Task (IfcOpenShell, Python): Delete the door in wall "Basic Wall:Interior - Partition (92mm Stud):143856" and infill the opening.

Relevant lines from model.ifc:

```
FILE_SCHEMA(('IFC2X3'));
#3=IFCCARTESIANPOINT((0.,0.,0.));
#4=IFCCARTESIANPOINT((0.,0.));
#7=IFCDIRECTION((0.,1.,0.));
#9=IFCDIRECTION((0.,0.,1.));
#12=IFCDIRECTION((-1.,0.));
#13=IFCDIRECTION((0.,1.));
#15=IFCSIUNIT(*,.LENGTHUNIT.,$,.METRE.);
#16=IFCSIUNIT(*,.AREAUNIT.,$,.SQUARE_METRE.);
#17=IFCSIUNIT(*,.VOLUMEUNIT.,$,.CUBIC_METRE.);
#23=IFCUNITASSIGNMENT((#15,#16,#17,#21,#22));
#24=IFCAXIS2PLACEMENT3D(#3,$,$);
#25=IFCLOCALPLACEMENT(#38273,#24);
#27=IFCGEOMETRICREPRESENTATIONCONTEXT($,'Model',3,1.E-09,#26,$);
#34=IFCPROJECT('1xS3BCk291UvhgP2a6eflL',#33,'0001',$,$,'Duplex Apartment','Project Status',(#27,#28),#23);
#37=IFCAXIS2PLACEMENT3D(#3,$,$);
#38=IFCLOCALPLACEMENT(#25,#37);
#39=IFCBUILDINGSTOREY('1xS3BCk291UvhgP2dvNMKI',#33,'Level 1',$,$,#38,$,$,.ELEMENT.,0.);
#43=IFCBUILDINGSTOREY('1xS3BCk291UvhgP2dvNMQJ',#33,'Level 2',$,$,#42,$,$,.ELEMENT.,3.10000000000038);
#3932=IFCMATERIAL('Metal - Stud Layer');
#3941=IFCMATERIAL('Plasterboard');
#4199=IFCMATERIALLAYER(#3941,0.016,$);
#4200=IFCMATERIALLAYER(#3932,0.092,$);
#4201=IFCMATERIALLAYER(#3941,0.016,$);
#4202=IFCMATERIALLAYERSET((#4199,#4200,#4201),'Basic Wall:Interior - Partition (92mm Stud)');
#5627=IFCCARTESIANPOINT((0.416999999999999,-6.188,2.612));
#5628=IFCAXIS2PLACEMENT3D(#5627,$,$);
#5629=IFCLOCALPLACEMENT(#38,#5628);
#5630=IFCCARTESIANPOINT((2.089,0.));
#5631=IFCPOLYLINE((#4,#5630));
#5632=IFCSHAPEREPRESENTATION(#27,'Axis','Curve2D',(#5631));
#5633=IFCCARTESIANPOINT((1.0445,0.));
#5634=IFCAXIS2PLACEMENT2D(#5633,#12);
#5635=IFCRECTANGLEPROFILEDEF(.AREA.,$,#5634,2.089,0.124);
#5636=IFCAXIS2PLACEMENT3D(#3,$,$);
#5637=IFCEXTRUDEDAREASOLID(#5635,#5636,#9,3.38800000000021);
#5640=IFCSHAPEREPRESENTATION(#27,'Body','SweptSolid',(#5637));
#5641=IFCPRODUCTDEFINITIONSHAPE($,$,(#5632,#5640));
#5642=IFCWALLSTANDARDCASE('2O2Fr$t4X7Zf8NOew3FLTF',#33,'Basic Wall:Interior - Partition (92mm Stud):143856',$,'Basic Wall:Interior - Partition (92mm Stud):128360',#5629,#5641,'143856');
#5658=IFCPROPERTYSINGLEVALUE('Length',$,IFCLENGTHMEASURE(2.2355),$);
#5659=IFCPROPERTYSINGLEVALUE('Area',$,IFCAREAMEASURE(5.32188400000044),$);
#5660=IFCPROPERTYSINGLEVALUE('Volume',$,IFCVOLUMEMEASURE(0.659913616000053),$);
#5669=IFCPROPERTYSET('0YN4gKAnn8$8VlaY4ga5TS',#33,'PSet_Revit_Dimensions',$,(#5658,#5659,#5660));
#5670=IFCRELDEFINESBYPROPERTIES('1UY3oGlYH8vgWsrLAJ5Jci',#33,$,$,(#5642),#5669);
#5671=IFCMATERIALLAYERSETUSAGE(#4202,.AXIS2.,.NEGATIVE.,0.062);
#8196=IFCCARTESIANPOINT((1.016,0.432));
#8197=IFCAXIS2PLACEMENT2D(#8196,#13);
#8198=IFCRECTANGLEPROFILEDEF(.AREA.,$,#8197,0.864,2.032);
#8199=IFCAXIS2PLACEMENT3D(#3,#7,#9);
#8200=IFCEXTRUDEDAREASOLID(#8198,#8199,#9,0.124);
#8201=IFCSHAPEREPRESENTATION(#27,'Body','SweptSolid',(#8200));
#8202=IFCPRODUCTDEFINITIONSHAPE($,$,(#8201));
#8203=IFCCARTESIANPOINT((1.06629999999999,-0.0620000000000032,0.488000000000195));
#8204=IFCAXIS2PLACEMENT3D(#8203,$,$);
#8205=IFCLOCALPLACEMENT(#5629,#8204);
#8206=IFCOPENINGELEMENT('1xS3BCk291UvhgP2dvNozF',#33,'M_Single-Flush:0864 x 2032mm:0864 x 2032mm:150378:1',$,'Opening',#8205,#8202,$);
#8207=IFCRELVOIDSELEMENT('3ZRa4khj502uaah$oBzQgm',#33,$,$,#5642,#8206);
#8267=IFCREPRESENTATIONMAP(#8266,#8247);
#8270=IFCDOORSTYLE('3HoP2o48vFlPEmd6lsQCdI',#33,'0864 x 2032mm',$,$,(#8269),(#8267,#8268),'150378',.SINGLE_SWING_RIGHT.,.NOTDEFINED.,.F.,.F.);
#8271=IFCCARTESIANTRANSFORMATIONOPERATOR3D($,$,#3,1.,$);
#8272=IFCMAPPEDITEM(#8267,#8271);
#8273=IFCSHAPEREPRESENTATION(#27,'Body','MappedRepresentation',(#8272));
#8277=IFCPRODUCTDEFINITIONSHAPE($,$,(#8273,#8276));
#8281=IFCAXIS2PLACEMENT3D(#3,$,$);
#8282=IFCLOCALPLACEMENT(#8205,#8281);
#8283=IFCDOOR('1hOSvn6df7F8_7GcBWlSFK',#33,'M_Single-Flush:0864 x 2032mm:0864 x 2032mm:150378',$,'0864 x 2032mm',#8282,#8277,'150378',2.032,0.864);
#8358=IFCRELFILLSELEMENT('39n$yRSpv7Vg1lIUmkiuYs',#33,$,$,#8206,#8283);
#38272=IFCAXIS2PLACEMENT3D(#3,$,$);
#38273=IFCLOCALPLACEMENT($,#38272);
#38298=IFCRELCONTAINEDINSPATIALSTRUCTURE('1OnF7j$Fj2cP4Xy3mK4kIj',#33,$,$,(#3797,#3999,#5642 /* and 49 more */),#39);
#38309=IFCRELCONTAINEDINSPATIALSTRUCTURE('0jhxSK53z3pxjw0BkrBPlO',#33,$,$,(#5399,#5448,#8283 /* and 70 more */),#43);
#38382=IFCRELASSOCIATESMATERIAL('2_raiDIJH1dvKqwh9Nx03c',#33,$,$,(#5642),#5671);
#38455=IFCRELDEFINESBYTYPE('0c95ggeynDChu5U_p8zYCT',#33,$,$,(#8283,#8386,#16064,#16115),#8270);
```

```python
import ifcopenshell
import ifcopenshell.api.feature
import ifcopenshell.api.pset
import ifcopenshell.api.root
import ifcopenshell.geom
import ifcopenshell.util.element
import ifcopenshell.util.shape
import ifcopenshell.util.unit

model = ifcopenshell.open("model.ifc")
area_scale = ifcopenshell.util.unit.calculate_unit_scale(model, "AREAUNIT")
volume_scale = ifcopenshell.util.unit.calculate_unit_scale(model, "VOLUMEUNIT")
settings = ifcopenshell.geom.settings()


def volume(element):
    """Net volume in cubic metres, openings subtracted."""
    shape = ifcopenshell.geom.create_shape(settings, element)
    return ifcopenshell.util.shape.get_volume(shape.geometry)


door = model.by_guid("1hOSvn6df7F8_7GcBWlSFK")
opening = door.FillsVoids[0].RelatingOpeningElement
wall = opening.VoidsElements[0].RelatingBuildingElement
before = volume(wall)

ifcopenshell.api.root.remove_product(model, product=door)
ifcopenshell.api.feature.remove_feature(model, feature=opening)

after = volume(wall)
thickness = 0.124  # wall thickness in metres

# Update the wall's stored quantities.
pset = model.by_id(ifcopenshell.util.element.get_pset(wall, "PSet_Revit_Dimensions", should_inherit=False)["id"])
ifcopenshell.api.pset.edit_pset(model, pset=pset, properties={
    "Area": model.create_entity("IfcAreaMeasure", after / thickness / area_scale),
    "Volume": model.create_entity("IfcVolumeMeasure", after / volume_scale),
})

print(f"wall volume {before:.3f} -> {after:.3f} m3")

model.write("model-out.ifc")
```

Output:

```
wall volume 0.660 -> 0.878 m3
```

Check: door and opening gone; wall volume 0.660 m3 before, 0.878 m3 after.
